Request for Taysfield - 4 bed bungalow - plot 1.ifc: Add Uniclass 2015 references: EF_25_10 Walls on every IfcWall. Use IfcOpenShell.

First a look at what the model holds.

```python
import ifcopenshell

model = ifcopenshell.open("Taysfield - 4 bed bungalow - plot 1.ifc")
print(model.schema)
print("classifications:", [c.Name for c in model.by_type("IfcClassification")])
for ifc_class in ("IfcDoor", "IfcRoof", "IfcStair", "IfcWall", "IfcWindow"):
    print(ifc_class, len(model.by_type(ifc_class)))
```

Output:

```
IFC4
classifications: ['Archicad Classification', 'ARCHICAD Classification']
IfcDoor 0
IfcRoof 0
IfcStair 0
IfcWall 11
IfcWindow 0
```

```python
import ifcopenshell
import ifcopenshell.api.classification

model = ifcopenshell.open("Taysfield - 4 bed bungalow - plot 1.ifc")

system = ifcopenshell.api.classification.add_classification(model, classification="Uniclass 2015")

codes = {
    "IfcWall": ("EF_25_10", "Walls"),
}
for ifc_class, (code, name) in codes.items():
    products = model.by_type(ifc_class)
    ifcopenshell.api.classification.add_reference(
        model, products=products, classification=system, identification=code, name=name
    )
    print(code, len(products))

model.write("Taysfield - 4 bed bungalow - plot 1-out.ifc")
```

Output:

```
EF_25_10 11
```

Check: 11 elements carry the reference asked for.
